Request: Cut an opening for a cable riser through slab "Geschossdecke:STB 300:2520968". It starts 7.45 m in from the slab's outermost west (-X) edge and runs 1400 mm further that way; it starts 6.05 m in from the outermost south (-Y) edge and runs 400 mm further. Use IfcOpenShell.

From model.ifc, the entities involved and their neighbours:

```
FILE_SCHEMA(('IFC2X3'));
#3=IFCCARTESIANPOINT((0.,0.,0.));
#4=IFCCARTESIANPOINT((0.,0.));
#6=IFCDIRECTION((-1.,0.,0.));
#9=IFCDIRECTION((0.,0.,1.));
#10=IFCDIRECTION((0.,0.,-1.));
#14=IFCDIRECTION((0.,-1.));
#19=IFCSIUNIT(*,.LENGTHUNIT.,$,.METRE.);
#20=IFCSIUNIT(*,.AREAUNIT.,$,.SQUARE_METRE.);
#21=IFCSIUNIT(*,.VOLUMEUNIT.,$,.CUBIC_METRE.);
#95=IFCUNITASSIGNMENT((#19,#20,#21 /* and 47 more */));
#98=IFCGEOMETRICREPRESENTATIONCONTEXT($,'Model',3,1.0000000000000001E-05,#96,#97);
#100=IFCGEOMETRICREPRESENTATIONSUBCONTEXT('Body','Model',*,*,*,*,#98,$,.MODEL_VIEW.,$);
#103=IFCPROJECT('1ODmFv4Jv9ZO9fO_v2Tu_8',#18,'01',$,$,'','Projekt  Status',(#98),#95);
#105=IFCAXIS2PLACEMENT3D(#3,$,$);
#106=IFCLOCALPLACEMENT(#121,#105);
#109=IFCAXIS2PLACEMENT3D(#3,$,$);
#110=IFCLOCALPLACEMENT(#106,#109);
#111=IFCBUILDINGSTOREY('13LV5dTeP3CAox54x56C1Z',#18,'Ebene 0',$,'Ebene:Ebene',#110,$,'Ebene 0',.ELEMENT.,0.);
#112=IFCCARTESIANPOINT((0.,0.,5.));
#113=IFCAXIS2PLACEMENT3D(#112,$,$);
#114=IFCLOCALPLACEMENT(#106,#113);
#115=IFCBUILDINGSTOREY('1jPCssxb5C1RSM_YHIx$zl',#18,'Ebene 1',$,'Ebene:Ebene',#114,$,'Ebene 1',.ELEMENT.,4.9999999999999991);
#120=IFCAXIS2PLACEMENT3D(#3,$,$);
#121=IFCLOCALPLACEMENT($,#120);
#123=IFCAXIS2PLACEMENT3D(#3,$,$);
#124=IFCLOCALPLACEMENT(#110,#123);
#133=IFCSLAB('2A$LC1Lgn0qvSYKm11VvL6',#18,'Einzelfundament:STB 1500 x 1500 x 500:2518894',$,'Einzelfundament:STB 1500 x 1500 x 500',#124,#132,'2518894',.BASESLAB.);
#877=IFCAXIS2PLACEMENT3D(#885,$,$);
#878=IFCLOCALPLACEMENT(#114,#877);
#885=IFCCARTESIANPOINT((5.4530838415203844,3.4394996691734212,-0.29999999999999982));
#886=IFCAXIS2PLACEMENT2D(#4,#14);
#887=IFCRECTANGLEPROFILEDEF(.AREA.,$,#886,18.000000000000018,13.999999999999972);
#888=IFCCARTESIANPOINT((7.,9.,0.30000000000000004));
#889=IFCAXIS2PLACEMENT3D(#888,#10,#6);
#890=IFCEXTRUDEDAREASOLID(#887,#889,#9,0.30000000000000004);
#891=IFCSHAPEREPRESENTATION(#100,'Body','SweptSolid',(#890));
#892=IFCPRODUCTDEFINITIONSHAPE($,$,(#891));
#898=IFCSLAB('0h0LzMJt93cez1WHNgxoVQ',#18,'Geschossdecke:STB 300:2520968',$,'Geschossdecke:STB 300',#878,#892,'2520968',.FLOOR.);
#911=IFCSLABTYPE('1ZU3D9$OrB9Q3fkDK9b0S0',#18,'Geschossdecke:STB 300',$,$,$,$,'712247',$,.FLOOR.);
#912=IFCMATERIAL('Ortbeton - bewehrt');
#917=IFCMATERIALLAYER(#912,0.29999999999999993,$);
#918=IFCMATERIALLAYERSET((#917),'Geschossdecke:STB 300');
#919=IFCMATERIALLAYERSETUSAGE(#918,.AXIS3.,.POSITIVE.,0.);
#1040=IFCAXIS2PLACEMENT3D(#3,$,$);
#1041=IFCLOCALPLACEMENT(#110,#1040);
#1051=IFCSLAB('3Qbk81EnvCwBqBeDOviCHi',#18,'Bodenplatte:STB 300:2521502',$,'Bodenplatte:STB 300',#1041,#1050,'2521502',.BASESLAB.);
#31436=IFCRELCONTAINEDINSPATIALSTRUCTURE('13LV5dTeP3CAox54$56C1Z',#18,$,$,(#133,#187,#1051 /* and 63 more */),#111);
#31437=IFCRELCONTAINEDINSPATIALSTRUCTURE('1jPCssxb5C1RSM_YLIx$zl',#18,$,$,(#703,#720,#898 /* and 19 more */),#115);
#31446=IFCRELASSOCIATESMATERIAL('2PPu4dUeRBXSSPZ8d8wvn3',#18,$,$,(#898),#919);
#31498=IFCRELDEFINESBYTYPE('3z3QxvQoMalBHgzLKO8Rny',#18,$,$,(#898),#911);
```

```python
import numpy as np
import ifcopenshell
import ifcopenshell.api.feature
import ifcopenshell.api.geometry
import ifcopenshell.api.root
import ifcopenshell.geom
import ifcopenshell.util.placement
import ifcopenshell.util.representation
import ifcopenshell.util.shape
import ifcopenshell.util.unit

model = ifcopenshell.open("model.ifc")
unit_scale = ifcopenshell.util.unit.calculate_unit_scale(model)
settings = ifcopenshell.geom.settings()


def volume(element):
    """Net volume in cubic metres, openings subtracted."""
    shape = ifcopenshell.geom.create_shape(settings, element)
    return ifcopenshell.util.shape.get_volume(shape.geometry)


slab = model.by_guid("0h0LzMJt93cez1WHNgxoVQ")
before = volume(slab)

# Extent in the slab's own axes, in metres. The edges named are its -X and -Y sides.
slab_shape = ifcopenshell.geom.create_shape(settings, slab)
vertices = ifcopenshell.util.shape.get_vertices(slab_shape.geometry)
x_min, y_min, bottom = vertices.min(axis=0)
top = vertices[:, 2].max()

opening = ifcopenshell.api.root.create_entity(model, ifc_class="IfcOpeningElement", name="Cable riser opening")
context = ifcopenshell.util.representation.get_context(model, "Model", "Body", "MODEL_VIEW")
width, depth = 1.4, 0.4
outline = [(0.0, 0.0), (width, 0.0), (width, depth), (0.0, depth), (0.0, 0.0)]
# Overshoot both faces by 50 mm so the cut is clean.
shape = ifcopenshell.api.geometry.add_slab_representation(
    model, context=context, depth=top - bottom + 0.1, polyline=outline
)
ifcopenshell.api.geometry.assign_representation(model, product=opening, representation=shape)

matrix = ifcopenshell.util.placement.get_local_placement(slab.ObjectPlacement)
matrix[:, 3] = matrix @ np.append(np.array([x_min + 7.45, y_min + 6.05, bottom - 0.05]) / unit_scale, 1.0)
ifcopenshell.api.geometry.edit_object_placement(model, product=opening, matrix=matrix, is_si=False)
ifcopenshell.api.feature.add_feature(model, feature=opening, element=slab)

after = volume(slab)

print(f"slab volume {before:.3f} -> {after:.3f} m3")

model.write("model-out.ifc")
```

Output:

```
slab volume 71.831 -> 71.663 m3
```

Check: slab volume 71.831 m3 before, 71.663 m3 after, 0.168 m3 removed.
